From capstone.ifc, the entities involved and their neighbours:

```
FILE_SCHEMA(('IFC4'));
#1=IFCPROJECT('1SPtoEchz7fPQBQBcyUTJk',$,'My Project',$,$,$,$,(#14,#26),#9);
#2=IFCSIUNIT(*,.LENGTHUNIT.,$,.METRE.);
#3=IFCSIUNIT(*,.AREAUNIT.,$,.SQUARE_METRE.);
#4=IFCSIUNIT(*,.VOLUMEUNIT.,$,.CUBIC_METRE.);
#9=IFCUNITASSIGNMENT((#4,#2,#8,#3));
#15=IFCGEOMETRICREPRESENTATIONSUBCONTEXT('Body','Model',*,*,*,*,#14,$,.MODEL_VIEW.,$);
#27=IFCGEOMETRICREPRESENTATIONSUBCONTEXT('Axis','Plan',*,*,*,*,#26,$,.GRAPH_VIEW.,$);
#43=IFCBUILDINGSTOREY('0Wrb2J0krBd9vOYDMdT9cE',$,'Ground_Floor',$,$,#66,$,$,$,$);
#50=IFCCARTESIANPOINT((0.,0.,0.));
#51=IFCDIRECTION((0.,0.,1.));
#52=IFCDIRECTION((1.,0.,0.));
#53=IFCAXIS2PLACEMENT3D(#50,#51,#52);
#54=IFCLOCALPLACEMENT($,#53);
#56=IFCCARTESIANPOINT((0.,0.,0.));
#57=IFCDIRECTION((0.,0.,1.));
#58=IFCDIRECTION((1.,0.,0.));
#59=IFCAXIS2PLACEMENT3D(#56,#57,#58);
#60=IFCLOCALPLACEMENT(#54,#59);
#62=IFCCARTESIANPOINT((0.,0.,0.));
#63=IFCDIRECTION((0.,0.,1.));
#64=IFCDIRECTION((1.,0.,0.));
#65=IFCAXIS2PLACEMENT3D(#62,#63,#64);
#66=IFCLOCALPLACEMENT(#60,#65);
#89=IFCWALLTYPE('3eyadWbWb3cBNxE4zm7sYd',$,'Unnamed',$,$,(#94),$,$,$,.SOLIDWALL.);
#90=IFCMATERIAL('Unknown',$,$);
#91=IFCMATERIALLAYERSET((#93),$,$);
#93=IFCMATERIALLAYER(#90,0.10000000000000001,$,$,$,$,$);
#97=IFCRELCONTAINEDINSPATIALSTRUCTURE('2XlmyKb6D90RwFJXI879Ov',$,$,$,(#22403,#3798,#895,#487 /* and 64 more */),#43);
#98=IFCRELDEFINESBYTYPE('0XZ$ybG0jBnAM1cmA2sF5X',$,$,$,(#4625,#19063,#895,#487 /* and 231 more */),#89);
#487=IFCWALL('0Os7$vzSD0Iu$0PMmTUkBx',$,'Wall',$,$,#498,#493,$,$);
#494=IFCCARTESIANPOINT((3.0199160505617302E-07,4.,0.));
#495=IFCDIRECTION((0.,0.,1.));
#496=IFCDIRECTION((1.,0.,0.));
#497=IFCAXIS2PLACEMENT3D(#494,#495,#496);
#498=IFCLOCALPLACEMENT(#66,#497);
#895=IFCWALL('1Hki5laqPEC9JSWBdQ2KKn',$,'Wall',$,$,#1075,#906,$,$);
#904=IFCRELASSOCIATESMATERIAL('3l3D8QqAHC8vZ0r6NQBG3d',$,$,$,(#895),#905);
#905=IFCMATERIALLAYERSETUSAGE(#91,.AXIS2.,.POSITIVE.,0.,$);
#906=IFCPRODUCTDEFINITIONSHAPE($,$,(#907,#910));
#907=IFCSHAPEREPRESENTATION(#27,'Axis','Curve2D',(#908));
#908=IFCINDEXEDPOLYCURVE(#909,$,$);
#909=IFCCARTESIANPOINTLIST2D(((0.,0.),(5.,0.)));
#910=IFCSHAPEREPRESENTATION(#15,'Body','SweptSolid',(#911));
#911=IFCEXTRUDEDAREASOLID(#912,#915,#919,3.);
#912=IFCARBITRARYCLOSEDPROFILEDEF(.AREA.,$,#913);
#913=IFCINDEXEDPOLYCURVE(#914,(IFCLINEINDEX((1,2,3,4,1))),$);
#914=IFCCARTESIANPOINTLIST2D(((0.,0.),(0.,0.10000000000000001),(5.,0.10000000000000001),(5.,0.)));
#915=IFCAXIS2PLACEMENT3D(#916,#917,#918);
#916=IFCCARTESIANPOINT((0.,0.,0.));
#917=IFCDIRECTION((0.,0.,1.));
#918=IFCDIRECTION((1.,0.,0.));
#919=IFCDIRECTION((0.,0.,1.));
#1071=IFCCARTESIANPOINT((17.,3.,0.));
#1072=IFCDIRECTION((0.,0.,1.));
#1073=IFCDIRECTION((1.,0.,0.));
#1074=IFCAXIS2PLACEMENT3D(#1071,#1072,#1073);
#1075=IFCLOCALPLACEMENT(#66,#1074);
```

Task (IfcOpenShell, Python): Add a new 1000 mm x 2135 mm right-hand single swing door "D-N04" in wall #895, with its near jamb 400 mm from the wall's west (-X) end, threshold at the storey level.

```python
import numpy as np
import ifcopenshell
import ifcopenshell.api.feature
import ifcopenshell.api.geometry
import ifcopenshell.api.root
import ifcopenshell.api.spatial
import ifcopenshell.geom
import ifcopenshell.util.element
import ifcopenshell.util.placement
import ifcopenshell.util.representation
import ifcopenshell.util.shape
import ifcopenshell.util.unit

model = ifcopenshell.open("capstone.ifc")
unit_scale = ifcopenshell.util.unit.calculate_unit_scale(model)
settings = ifcopenshell.geom.settings()


def volume(element):
    """Net volume in cubic metres, openings subtracted."""
    shape = ifcopenshell.geom.create_shape(settings, element)
    return ifcopenshell.util.shape.get_volume(shape.geometry)


wall = model.by_guid("1Hki5laqPEC9JSWBdQ2KKn")
storey = ifcopenshell.util.element.get_container(wall, ifc_class="IfcBuildingStorey")
context = ifcopenshell.util.representation.get_context(model, "Model", "Body", "MODEL_VIEW")
before = volume(wall)

width, height, from_end, sill = 1, 2.135, 0.4, 0.0  # metres

# The wall runs along its own X axis, and the end named is its -X end.
wall_shape = ifcopenshell.geom.create_shape(settings, wall)
x, y, z = ifcopenshell.util.shape.get_vertices(wall_shape.geometry).T
start = x.min() + from_end
face, thickness = float(y.min()), float(y.max() - y.min())
wall_matrix = ifcopenshell.util.placement.get_local_placement(wall.ObjectPlacement)
level = ifcopenshell.util.placement.get_local_placement(storey.ObjectPlacement)[2, 3]


def in_wall(x, y):
    """Placement at x, y metres in the wall's axes, at sill height."""
    matrix = wall_matrix.copy()
    matrix[:, 3] = wall_matrix @ np.array([x / unit_scale, y / unit_scale, 0.0, 1.0])
    matrix[2, 3] = level + sill / unit_scale
    return matrix


# Opening: a box that overshoots both wall faces by 50 mm.
opening = ifcopenshell.api.root.create_entity(model, ifc_class="IfcOpeningElement", predefined_type="OPENING")
box = ifcopenshell.api.geometry.add_wall_representation(
    model, context=context, length=width, height=height, thickness=thickness + 0.1
)
ifcopenshell.api.geometry.assign_representation(model, product=opening, representation=box)
ifcopenshell.api.geometry.edit_object_placement(model, product=opening, matrix=in_wall(start, face - 0.05), is_si=False)
ifcopenshell.api.feature.add_feature(model, feature=opening, element=wall)

door = ifcopenshell.api.root.create_entity(model, ifc_class="IfcDoor", name="D-N04", predefined_type="DOOR")
door.OverallWidth, door.OverallHeight = width / unit_scale, height / unit_scale
door.OperationType = "SINGLE_SWING_RIGHT"
body = ifcopenshell.api.geometry.add_door_representation(
    model,
    context=context,
    overall_width=door.OverallWidth,
    overall_height=door.OverallHeight,
    operation_type="SINGLE_SWING_RIGHT",
    lining_properties={"LiningDepth": thickness / unit_scale, "ThresholdDepth": thickness / unit_scale},
)
ifcopenshell.api.geometry.assign_representation(model, product=door, representation=body)
ifcopenshell.api.spatial.assign_container(model, products=[door], relating_structure=storey)
ifcopenshell.api.feature.add_filling(model, opening=opening, element=door)

# The lining spans the wall, so the door starts at the wall face.
ifcopenshell.api.geometry.edit_object_placement(model, product=door, matrix=in_wall(start, face), is_si=False)

after = volume(wall)

print(f"wall volume {before:.3f} -> {after:.3f} m3")

model.write("capstone_v2.ifc")
```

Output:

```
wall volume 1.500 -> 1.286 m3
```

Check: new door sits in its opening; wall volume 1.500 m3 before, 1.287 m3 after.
